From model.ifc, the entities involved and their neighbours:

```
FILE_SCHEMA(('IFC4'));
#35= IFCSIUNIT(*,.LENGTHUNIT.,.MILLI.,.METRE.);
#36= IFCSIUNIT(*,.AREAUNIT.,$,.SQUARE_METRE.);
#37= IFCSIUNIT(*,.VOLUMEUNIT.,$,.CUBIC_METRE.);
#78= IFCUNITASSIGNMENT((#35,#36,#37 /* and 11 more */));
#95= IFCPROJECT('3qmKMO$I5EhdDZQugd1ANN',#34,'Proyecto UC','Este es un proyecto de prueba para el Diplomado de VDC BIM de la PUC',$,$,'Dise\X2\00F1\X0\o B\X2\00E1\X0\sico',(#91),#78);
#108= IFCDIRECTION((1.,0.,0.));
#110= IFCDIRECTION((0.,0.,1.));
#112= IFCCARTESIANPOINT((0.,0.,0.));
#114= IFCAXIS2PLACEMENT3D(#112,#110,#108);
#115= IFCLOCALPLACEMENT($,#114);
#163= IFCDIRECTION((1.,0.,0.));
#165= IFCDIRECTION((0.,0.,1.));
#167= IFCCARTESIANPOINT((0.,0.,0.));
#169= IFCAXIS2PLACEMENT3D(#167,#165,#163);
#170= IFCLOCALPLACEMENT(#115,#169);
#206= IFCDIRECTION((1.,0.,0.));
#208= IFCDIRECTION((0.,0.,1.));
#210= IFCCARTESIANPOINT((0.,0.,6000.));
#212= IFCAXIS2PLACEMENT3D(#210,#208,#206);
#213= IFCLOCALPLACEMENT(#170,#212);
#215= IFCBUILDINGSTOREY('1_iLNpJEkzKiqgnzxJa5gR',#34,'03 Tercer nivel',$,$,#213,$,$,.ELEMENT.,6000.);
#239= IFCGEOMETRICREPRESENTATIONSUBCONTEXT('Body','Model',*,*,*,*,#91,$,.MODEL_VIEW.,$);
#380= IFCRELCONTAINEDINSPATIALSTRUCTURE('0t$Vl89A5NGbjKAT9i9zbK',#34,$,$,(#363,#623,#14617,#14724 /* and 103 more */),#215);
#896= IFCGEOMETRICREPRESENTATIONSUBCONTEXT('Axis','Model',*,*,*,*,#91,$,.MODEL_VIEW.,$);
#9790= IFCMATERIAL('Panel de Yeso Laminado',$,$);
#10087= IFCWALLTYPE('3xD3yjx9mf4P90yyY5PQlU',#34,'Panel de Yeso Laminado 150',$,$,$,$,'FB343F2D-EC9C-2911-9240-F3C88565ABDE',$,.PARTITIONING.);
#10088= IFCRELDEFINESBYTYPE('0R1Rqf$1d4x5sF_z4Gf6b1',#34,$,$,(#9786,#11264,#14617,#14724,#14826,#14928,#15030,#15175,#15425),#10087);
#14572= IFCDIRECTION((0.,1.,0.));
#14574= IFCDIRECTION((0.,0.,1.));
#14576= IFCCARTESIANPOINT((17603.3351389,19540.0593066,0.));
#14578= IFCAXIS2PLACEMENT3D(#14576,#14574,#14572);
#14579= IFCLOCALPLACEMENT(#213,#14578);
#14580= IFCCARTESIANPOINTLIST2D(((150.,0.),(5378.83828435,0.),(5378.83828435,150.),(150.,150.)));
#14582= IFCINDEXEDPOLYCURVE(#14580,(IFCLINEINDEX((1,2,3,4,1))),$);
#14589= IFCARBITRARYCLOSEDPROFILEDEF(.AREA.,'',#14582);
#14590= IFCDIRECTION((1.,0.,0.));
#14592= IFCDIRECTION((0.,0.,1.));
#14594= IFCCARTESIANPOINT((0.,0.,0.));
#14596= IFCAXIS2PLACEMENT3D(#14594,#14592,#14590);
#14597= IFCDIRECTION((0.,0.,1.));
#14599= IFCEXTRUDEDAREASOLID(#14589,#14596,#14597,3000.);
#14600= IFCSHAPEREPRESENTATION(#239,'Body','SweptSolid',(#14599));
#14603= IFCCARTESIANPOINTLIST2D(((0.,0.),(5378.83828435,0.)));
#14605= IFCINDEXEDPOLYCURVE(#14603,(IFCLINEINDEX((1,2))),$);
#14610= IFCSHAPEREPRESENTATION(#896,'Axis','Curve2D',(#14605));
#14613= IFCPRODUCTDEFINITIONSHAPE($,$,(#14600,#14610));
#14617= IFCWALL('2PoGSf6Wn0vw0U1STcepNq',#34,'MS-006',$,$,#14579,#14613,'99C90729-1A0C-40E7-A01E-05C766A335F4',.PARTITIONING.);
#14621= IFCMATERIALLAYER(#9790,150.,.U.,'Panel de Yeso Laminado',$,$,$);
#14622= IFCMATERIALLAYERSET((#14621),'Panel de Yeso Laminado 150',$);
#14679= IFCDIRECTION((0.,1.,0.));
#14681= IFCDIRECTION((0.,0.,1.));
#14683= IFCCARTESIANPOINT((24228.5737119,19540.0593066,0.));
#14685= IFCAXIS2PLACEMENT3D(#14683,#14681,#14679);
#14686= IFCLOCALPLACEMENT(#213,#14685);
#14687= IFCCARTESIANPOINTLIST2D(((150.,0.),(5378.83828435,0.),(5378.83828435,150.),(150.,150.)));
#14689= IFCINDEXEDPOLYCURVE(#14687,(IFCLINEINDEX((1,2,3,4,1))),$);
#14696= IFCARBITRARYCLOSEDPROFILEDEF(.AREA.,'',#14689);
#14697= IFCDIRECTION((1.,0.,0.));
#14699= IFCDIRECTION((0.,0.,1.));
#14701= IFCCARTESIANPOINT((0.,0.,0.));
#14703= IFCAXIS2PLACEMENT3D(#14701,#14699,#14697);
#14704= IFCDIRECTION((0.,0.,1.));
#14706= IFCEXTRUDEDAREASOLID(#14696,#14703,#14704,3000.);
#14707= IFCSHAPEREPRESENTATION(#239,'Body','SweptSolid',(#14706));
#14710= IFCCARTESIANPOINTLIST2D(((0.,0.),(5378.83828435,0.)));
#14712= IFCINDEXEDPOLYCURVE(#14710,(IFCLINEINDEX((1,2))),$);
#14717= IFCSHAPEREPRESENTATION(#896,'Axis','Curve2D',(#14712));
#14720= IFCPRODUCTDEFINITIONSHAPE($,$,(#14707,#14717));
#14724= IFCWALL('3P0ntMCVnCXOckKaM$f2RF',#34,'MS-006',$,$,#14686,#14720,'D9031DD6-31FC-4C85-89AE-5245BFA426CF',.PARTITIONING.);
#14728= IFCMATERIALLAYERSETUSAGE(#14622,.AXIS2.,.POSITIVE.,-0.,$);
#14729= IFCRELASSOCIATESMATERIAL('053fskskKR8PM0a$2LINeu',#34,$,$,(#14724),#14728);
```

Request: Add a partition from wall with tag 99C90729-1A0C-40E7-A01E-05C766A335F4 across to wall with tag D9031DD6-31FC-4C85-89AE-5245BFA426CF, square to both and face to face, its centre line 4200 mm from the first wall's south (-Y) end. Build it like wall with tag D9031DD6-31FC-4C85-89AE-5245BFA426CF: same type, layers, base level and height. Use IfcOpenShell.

```python
import numpy as np
import ifcopenshell
import ifcopenshell.api.geometry
import ifcopenshell.api.material
import ifcopenshell.api.pset
import ifcopenshell.api.root
import ifcopenshell.api.spatial
import ifcopenshell.api.type
import ifcopenshell.geom
import ifcopenshell.util.element
import ifcopenshell.util.placement
import ifcopenshell.util.representation
import ifcopenshell.util.shape
import ifcopenshell.util.unit

model = ifcopenshell.open("model.ifc")
unit_scale = ifcopenshell.util.unit.calculate_unit_scale(model)
settings = ifcopenshell.geom.settings()
settings.set("use-world-coords", True)

start_wall = model.by_guid("2PoGSf6Wn0vw0U1STcepNq")
end_wall = model.by_guid("3P0ntMCVnCXOckKaM$f2RF")
like = model.by_id(14724)
matrix = ifcopenshell.util.placement.get_local_placement(start_wall.ObjectPlacement)
matrix[:3, 3] *= unit_scale


def extent(element):
    """Bounding box in the first wall's axes, in metres."""
    shape = ifcopenshell.geom.create_shape(settings, element)
    points = (ifcopenshell.util.shape.get_vertices(shape.geometry) - matrix[:3, 3]) @ matrix[:3, :3]
    return points.min(axis=0), points.max(axis=0)


y_start = extent(start_wall)[0][1]
y_end = extent(end_wall)[1][1]
like_min, like_max = extent(like)
length, height = float(abs(y_end - y_start)), float(like_max[2] - like_min[2])
layer_set = ifcopenshell.util.element.get_material(like, should_skip_usage=True)
thickness = sum(layer.LayerThickness for layer in layer_set.MaterialLayers) * unit_scale

wall = ifcopenshell.api.root.create_entity(model, ifc_class="IfcWall", name="New partition")
storey = ifcopenshell.util.element.get_container(like)
ifcopenshell.api.spatial.assign_container(model, products=[wall], relating_structure=storey)
ifcopenshell.api.type.assign_type(
    model, related_objects=[wall], relating_type=ifcopenshell.util.element.get_type(like), should_map_representations=False
)
rel = ifcopenshell.api.material.assign_material(
    model, products=[wall], type="IfcMaterialLayerSetUsage", material=layer_set
)
rel.RelatingMaterial.OffsetFromReferenceLine = -thickness / 2 / unit_scale
pset = ifcopenshell.api.pset.add_pset(model, product=wall, name="Pset_WallCommon")
ifcopenshell.api.pset.edit_pset(model, pset=pset, properties={"IsExternal": False, "LoadBearing": False})

# The axis runs down the middle of the wall.
axis = ifcopenshell.api.geometry.add_axis_representation(
    model, context=ifcopenshell.util.representation.get_context(model, "Model", "Axis"), axis=[(0.0, 0.0), (length, 0.0)]
)
body = ifcopenshell.api.geometry.add_wall_representation(
    model,
    context=ifcopenshell.util.representation.get_context(model, "Model", "Body", "MODEL_VIEW"),
    length=length,
    height=height,
    thickness=thickness,
    offset=-thickness / 2,
)
for representation in (axis, body):
    ifcopenshell.api.geometry.assign_representation(model, product=wall, representation=representation)

placement = matrix @ ifcopenshell.util.placement.rotation(-90, "Z")
placement[:, 3] = matrix @ np.array([extent(start_wall)[0][0] + 4.2, y_start, like_min[2], 1.0])
ifcopenshell.api.geometry.edit_object_placement(model, product=wall, matrix=placement)

print(f"partition {length:.3f} m long, {height:.3f} m high, {thickness:.3f} m thick")

model.write("model_updated.ifc")
```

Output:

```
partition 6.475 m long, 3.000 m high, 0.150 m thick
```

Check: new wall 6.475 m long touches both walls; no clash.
